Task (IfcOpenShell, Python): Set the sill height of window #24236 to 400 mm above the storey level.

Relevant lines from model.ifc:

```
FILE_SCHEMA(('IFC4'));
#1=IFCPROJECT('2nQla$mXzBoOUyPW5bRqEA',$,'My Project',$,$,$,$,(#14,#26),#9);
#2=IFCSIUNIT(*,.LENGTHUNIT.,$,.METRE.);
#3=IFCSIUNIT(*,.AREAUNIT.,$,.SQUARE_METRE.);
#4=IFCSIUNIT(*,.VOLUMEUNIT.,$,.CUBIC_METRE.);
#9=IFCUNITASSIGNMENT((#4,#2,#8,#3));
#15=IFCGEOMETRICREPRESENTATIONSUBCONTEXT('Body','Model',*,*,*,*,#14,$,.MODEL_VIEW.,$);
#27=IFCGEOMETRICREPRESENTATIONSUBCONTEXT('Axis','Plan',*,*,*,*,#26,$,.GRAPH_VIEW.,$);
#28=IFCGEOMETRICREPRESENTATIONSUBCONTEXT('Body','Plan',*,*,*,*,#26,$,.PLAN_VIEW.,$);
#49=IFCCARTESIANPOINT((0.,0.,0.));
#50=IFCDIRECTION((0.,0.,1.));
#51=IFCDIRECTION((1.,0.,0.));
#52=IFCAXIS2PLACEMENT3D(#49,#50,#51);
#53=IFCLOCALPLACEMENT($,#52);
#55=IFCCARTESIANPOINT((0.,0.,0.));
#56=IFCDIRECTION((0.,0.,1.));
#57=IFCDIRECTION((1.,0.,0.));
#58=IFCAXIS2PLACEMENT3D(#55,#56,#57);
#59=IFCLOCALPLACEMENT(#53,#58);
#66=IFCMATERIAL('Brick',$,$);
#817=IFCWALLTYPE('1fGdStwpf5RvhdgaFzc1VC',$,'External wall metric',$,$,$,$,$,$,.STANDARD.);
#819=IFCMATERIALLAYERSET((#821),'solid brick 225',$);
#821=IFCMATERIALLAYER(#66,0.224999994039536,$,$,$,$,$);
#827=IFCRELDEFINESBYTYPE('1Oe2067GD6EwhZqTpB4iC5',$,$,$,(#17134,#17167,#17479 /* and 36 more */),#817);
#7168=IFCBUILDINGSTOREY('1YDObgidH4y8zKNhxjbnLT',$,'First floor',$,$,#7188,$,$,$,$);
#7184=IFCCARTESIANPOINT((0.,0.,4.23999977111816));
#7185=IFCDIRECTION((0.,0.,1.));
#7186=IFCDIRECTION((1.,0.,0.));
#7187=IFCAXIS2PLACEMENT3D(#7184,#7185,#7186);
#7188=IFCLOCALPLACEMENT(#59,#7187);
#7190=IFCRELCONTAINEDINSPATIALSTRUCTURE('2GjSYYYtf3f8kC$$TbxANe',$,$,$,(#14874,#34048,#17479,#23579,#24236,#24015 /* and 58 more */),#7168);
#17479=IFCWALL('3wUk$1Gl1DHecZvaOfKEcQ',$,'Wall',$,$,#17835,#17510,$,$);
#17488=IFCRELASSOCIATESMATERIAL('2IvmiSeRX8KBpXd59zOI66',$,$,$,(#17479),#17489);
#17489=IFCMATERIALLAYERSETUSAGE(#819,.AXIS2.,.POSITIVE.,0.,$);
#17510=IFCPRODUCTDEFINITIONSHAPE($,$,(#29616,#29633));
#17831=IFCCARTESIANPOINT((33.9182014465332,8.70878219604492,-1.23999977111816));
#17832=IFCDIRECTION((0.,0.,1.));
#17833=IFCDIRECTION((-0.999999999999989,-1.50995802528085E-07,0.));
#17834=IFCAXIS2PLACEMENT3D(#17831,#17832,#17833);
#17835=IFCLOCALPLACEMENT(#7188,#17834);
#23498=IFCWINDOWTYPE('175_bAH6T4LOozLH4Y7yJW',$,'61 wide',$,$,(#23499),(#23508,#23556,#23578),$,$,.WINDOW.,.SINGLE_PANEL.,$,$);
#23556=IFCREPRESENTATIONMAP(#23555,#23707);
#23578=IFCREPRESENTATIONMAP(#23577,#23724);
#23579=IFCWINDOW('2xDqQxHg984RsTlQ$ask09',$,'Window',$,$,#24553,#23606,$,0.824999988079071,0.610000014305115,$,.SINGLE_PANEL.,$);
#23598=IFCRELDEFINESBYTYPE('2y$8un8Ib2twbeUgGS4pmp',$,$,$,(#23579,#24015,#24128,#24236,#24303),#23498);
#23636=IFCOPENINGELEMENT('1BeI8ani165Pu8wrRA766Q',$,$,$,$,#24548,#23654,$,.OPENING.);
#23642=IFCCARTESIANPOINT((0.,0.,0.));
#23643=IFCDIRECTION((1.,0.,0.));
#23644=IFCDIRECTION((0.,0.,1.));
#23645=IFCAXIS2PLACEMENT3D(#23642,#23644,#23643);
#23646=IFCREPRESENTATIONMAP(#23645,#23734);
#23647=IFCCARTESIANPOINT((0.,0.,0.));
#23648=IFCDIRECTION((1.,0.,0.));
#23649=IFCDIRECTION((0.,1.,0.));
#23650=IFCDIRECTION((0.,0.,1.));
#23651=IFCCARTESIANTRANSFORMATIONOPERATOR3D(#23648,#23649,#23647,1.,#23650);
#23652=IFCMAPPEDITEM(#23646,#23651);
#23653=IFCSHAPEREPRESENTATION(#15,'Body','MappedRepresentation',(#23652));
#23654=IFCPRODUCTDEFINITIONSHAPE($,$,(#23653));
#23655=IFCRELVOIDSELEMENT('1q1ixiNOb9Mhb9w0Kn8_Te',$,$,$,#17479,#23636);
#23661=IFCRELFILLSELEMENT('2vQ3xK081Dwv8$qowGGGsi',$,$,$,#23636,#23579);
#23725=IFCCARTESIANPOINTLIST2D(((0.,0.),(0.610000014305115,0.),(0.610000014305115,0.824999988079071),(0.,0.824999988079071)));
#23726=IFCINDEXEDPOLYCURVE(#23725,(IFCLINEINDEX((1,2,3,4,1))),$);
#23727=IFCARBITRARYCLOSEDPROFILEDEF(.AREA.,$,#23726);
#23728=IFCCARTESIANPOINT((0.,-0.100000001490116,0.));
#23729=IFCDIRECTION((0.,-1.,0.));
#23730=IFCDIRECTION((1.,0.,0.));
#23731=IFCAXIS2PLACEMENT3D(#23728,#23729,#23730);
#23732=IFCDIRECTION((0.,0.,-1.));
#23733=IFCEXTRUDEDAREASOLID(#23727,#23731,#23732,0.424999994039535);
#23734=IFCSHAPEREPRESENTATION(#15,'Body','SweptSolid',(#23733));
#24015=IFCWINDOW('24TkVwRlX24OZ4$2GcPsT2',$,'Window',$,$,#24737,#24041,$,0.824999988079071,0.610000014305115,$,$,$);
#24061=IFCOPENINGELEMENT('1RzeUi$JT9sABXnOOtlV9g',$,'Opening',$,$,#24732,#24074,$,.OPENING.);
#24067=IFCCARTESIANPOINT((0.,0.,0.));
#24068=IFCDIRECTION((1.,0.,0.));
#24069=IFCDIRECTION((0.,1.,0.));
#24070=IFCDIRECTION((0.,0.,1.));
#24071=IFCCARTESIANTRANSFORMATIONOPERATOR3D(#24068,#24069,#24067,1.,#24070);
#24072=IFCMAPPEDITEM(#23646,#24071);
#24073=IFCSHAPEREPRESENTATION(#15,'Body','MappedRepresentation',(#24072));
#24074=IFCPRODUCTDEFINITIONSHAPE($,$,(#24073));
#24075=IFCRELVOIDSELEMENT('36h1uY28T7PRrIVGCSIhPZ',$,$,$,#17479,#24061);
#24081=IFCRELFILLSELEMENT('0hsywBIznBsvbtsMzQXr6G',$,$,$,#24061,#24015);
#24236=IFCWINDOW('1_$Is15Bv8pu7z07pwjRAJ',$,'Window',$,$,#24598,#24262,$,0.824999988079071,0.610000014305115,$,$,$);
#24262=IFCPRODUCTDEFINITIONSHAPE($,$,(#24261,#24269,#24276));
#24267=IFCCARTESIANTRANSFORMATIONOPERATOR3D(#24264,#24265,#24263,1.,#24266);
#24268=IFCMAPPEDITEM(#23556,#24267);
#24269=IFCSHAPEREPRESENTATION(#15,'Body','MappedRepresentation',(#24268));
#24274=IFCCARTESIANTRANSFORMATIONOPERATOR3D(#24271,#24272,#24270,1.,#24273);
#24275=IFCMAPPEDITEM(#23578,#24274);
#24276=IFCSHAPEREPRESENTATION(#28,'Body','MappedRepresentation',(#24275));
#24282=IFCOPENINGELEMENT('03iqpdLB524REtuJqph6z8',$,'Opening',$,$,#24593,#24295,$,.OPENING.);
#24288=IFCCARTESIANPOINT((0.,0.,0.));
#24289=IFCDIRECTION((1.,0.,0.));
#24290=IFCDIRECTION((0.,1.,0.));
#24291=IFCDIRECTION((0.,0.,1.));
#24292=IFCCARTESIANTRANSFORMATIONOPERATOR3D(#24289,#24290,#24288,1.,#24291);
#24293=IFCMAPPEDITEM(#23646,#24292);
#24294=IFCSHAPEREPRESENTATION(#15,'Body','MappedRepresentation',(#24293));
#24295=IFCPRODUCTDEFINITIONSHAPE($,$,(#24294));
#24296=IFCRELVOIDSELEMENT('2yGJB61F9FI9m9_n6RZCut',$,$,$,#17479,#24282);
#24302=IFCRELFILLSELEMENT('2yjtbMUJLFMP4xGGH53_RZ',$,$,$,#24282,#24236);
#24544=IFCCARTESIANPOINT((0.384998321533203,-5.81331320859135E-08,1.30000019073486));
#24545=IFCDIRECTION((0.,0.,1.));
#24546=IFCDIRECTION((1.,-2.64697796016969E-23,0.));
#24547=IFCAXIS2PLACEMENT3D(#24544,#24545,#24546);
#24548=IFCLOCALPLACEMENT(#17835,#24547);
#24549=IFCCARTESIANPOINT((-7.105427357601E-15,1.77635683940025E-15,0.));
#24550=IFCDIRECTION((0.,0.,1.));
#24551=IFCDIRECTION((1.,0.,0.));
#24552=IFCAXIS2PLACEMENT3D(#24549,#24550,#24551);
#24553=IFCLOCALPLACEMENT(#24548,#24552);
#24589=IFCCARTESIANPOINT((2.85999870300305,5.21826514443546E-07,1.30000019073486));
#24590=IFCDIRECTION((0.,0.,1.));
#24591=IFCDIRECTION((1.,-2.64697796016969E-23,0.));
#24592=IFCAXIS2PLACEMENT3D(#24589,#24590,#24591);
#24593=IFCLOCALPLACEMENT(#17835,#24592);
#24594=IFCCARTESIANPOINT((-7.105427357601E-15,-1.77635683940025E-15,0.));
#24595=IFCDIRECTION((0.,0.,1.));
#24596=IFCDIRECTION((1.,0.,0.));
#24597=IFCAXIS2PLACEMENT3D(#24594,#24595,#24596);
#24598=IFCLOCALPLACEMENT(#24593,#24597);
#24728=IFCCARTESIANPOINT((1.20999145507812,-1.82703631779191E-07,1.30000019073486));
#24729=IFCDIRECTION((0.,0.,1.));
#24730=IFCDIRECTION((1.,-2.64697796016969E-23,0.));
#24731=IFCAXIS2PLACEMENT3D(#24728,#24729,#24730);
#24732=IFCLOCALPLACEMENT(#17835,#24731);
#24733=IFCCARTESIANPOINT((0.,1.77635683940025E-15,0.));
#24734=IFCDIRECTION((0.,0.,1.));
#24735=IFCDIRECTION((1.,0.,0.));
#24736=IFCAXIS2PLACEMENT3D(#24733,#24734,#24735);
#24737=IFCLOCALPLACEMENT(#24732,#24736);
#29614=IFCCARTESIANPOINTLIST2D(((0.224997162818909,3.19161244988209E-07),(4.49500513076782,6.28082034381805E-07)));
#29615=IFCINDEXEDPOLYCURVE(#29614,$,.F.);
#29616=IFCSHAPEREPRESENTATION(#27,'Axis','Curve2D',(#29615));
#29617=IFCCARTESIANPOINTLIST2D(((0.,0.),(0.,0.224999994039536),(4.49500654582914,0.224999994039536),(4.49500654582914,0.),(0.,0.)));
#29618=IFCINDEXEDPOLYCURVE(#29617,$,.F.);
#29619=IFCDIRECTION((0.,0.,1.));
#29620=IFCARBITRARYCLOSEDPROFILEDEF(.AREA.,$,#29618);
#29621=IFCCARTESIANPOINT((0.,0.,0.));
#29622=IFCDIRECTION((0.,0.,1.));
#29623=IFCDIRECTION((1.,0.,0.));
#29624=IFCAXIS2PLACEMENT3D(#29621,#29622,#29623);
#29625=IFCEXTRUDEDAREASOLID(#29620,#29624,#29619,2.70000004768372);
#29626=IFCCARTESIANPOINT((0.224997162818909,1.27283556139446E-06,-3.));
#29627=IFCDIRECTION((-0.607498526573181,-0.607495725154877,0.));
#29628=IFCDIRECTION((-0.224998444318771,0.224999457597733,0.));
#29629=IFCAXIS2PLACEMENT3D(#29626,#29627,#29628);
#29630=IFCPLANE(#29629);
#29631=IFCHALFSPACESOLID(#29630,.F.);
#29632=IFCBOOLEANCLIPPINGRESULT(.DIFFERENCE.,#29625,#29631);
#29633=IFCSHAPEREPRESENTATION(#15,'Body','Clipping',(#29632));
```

```python
import numpy as np
import ifcopenshell
import ifcopenshell.api.geometry
import ifcopenshell.geom
import ifcopenshell.util.element
import ifcopenshell.util.placement
import ifcopenshell.util.shape
import ifcopenshell.util.unit

model = ifcopenshell.open("model.ifc")
unit_scale = ifcopenshell.util.unit.calculate_unit_scale(model)

window = model.by_id(24236)
opening = window.FillsVoids[0].RelatingOpeningElement
storey = ifcopenshell.util.element.get_container(window, ifc_class="IfcBuildingStorey")
level = ifcopenshell.util.placement.get_local_placement(storey.ObjectPlacement)[2, 3]

# The opening's origin need not be at the sill, so measure its lowest point.
shape = ifcopenshell.geom.create_shape(ifcopenshell.geom.settings(), opening)
bottom = ifcopenshell.util.shape.get_shape_bottom_elevation(shape, shape.geometry) / unit_scale
dz = level + 0.4 - bottom

shift = np.array([0.0, 0.0, dz])
# The window is placed relative to its opening, so it follows when the opening moves.
matrix = ifcopenshell.util.placement.get_local_placement(opening.ObjectPlacement)
matrix[:3, 3] += shift
ifcopenshell.api.geometry.edit_object_placement(
    model, product=opening, matrix=matrix, is_si=False, should_transform_children=True
)

print(f"moved by {dz * unit_scale:+.3f} m")

model.write("model_v2.ifc")
```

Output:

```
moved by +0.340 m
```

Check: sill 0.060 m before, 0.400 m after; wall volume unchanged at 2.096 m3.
